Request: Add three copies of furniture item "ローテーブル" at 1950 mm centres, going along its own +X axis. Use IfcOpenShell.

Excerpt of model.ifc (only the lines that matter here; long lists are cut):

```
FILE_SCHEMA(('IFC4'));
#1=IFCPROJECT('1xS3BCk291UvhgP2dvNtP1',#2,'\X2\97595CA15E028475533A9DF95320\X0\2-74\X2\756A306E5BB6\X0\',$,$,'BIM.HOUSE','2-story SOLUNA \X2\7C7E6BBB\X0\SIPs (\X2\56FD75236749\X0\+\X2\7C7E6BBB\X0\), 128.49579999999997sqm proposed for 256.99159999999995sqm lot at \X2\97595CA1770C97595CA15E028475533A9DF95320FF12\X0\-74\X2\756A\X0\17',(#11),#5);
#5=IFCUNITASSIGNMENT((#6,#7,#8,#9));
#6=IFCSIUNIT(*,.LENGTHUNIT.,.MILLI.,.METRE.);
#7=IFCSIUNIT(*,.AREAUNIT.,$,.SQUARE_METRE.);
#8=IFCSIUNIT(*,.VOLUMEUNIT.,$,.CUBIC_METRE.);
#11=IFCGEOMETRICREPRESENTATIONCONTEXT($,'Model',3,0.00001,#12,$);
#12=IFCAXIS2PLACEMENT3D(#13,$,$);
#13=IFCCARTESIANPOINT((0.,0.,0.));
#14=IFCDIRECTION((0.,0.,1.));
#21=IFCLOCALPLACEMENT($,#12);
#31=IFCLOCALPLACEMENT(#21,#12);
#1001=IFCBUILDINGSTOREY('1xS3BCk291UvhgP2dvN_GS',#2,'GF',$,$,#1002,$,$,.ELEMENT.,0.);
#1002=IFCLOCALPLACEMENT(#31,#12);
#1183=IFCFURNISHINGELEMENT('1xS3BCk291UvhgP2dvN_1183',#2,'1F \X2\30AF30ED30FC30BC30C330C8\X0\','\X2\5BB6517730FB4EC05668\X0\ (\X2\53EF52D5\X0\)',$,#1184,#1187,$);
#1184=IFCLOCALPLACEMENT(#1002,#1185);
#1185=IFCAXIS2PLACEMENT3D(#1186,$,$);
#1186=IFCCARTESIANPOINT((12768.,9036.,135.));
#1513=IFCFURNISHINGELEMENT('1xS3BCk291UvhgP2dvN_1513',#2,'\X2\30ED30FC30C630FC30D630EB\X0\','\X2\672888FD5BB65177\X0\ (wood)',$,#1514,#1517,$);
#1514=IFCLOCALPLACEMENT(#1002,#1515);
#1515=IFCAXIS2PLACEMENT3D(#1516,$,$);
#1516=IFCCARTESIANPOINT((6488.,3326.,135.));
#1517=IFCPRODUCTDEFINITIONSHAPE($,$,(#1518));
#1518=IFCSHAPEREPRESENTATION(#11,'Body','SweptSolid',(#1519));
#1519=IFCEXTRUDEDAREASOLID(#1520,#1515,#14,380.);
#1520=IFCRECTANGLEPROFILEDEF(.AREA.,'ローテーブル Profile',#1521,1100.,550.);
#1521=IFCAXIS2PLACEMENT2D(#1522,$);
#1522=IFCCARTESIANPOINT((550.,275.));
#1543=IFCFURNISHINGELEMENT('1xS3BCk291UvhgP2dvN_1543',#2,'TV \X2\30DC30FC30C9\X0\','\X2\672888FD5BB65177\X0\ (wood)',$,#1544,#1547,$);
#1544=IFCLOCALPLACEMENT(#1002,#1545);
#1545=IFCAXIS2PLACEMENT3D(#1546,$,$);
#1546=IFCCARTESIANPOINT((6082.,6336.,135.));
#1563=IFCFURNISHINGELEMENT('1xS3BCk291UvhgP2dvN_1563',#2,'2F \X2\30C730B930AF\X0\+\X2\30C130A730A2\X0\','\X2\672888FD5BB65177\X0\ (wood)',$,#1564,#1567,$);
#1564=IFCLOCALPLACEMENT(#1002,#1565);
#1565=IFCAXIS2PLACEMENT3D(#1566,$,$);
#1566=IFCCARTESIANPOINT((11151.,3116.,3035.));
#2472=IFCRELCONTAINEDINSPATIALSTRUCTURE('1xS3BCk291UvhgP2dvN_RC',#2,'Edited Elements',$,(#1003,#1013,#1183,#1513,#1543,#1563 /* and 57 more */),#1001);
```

```python
import ifcopenshell
import ifcopenshell.api.geometry
import ifcopenshell.api.root
import ifcopenshell.util.element
import ifcopenshell.util.placement
import ifcopenshell.util.unit

model = ifcopenshell.open("model.ifc")
unit_scale = ifcopenshell.util.unit.calculate_unit_scale(model)


def reuse_history(source, copy):
    """copy_class also copies each property set's owner history, people and application; keep the originals."""
    for rel in copy.IsDefinedBy:
        if rel.is_a("IfcRelDefinesByProperties") and (history := rel.RelatingPropertyDefinition.OwnerHistory):
            rel.RelatingPropertyDefinition.OwnerHistory = source.OwnerHistory
            ifcopenshell.util.element.remove_deep2(model, history)


source = model.by_id(1513)
base = ifcopenshell.util.placement.get_local_placement(source.ObjectPlacement)
step = base[:3, 0] * 1.95 / unit_scale

for i in range(1, 4):
    copy = ifcopenshell.api.root.copy_class(model, product=source)
    copy.Representation = ifcopenshell.util.element.copy_deep(
        model, source.Representation, exclude=["IfcGeometricRepresentationContext", "IfcRepresentationMap"]
    )
    reuse_history(source, copy)
    matrix = base.copy()
    matrix[:3, 3] += i * step
    print("added at", matrix[:3, 3].round(3) + 0.0)
    ifcopenshell.api.geometry.edit_object_placement(model, product=copy, matrix=matrix, is_si=False)

model.write("model_v2.ifc")
```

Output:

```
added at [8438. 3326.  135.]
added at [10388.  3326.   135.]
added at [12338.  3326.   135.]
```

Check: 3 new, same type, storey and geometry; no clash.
